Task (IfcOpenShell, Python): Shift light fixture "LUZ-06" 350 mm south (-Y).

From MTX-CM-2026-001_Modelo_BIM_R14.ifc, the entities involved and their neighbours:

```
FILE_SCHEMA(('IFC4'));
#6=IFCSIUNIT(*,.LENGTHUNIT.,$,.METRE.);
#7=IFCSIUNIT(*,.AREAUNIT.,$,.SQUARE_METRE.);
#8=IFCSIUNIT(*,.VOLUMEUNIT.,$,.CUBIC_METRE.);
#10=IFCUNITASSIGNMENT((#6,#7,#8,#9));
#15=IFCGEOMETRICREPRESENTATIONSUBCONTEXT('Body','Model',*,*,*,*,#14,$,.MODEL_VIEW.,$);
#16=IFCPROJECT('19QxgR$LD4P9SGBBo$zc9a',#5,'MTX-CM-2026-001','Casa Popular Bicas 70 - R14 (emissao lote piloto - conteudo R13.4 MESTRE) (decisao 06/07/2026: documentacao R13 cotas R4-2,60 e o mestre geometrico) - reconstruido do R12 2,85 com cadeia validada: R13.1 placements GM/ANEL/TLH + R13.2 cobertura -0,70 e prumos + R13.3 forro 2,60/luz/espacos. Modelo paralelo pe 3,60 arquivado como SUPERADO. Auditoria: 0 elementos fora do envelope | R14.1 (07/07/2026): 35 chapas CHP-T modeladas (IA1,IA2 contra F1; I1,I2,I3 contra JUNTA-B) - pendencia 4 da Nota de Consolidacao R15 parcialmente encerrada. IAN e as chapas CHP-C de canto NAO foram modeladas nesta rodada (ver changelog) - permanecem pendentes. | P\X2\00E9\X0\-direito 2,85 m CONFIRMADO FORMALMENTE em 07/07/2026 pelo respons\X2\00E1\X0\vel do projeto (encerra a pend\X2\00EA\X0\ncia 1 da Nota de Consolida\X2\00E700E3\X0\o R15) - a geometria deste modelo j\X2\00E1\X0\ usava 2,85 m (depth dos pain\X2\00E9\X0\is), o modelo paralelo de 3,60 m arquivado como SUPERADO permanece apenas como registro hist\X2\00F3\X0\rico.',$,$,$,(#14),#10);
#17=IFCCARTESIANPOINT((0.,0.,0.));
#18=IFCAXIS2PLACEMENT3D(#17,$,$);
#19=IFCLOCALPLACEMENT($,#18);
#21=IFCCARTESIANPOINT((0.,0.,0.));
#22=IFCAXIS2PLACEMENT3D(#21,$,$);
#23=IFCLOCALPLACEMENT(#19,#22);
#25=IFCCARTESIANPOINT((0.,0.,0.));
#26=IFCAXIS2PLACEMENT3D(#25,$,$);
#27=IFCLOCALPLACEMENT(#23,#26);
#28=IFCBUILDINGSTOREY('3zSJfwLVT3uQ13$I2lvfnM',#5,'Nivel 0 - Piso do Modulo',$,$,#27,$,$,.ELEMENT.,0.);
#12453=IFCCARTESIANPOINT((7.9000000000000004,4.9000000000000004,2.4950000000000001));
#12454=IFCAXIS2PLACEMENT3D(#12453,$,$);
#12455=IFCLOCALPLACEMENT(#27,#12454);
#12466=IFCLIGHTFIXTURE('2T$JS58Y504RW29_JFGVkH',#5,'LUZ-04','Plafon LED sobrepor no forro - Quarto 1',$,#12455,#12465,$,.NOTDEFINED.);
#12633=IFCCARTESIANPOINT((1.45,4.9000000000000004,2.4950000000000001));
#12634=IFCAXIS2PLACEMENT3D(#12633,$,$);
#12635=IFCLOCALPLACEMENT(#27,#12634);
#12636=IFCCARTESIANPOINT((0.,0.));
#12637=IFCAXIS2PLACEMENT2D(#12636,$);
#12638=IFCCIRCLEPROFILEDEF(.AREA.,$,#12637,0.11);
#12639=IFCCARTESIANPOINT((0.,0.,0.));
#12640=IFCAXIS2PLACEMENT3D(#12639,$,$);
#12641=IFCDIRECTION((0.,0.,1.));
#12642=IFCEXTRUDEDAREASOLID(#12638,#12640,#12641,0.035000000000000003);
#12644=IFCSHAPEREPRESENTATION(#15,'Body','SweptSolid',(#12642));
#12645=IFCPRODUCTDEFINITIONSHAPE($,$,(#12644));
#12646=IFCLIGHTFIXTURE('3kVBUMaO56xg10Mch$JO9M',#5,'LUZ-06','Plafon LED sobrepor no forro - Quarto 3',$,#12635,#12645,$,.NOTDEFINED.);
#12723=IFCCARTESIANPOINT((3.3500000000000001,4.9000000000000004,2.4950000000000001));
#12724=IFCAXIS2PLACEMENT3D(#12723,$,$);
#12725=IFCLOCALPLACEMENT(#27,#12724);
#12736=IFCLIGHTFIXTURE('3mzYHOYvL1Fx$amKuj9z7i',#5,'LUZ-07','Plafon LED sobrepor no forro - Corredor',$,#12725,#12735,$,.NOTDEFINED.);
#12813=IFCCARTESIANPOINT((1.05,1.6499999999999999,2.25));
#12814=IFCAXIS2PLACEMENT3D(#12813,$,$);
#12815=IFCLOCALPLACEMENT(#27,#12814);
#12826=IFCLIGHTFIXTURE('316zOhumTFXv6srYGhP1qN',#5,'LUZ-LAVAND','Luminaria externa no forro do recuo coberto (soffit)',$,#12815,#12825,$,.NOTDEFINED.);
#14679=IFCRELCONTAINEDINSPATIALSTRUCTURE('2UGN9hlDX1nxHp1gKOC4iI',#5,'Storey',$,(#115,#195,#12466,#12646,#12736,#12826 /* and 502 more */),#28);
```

```python
import ifcopenshell
import ifcopenshell.api.geometry
import ifcopenshell.util.placement
import ifcopenshell.util.unit

model = ifcopenshell.open("MTX-CM-2026-001_Modelo_BIM_R14.ifc")
unit_scale = ifcopenshell.util.unit.calculate_unit_scale(model)

item = model.by_guid("3kVBUMaO56xg10Mch$JO9M")
matrix = ifcopenshell.util.placement.get_local_placement(item.ObjectPlacement)
matrix[1, 3] -= 0.35 / unit_scale
ifcopenshell.api.geometry.edit_object_placement(model, product=item, matrix=matrix, is_si=False)

print(ifcopenshell.util.placement.get_local_placement(item.ObjectPlacement).round(3) + 0.0)

model.write("MTX-CM-2026-001_Modelo_BIM_R14_updated.ifc")
```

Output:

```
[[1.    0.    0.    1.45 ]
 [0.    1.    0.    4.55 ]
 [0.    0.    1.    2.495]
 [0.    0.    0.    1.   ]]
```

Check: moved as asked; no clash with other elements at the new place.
